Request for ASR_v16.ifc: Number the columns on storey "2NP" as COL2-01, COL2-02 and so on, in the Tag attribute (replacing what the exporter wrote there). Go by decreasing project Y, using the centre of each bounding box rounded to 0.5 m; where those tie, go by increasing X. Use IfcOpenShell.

First a look at what the model holds.

```python
import ifcopenshell
import ifcopenshell.util.element
import ifcopenshell.util.placement

model = ifcopenshell.open("ASR_v16.ifc")
print(model.schema)
storey = next(s for s in model.by_type("IfcBuildingStorey") if s.Name == "2NP")
columns = [e for e in ifcopenshell.util.element.get_decomposition(storey) if e.is_a("IfcColumn")]
for e in sorted(columns, key=lambda e: e.id()):
    origin = ifcopenshell.util.placement.get_local_placement(e.ObjectPlacement)[:3, 3]
    print(e.id(), e.Tag, e.Name, origin.round(2) + 0.0, sep=" | ")
```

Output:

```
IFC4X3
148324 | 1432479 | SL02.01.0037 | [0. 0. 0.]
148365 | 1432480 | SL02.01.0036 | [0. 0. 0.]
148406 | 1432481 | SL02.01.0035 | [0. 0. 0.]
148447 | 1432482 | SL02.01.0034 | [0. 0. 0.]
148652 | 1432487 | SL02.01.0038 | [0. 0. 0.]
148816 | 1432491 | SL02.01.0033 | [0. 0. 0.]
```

```python
import ifcopenshell
import ifcopenshell.geom
import ifcopenshell.util.element
import ifcopenshell.util.shape

model = ifcopenshell.open("ASR_v16.ifc")
settings = ifcopenshell.geom.settings()
settings.set("use-world-coords", True)


def centre(element):
    shape = ifcopenshell.geom.create_shape(settings, element)
    return ifcopenshell.util.shape.get_bbox_centroid(shape.geometry)


storey = next(s for s in model.by_type("IfcBuildingStorey") if s.Name == "2NP")
columns = [e for e in ifcopenshell.util.element.get_decomposition(storey) if e.is_a("IfcColumn")]

# Insertion points can sit at a corner or the storey origin, so sort by the geometry (in metres).
centres = {e: centre(e) for e in columns}
columns.sort(key=lambda e: (-round(centres[e][1] / 0.5), centres[e][0]))

for i, e in enumerate(columns, start=1):
    number = f"COL2-{i:02d}"
    e.Tag = number
    print(e.id(), number)

model.write("ASR_v16-out.ifc")
```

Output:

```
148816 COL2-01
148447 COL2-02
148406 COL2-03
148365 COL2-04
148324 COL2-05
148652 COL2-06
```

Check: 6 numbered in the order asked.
